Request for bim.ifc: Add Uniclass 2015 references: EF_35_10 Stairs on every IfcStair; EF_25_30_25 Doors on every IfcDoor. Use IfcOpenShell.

First a look at what the model holds.

```python
import ifcopenshell

model = ifcopenshell.open("bim.ifc")
print(model.schema)
print("classifications:", [c.Name for c in model.by_type("IfcClassification")])
for ifc_class in ("IfcDoor", "IfcRoof", "IfcStair", "IfcWall", "IfcWindow"):
    print(ifc_class, len(model.by_type(ifc_class)))
```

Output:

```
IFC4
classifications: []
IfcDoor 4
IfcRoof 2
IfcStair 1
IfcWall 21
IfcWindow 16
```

```python
import ifcopenshell
import ifcopenshell.api.classification

model = ifcopenshell.open("bim.ifc")

system = ifcopenshell.api.classification.add_classification(model, classification="Uniclass 2015")

codes = {
    "IfcStair": ("EF_35_10", "Stairs"),
    "IfcDoor": ("EF_25_30_25", "Doors"),
}
for ifc_class, (code, name) in codes.items():
    products = model.by_type(ifc_class)
    ifcopenshell.api.classification.add_reference(
        model, products=products, classification=system, identification=code, name=name
    )
    print(code, len(products))

model.write("bim_updated.ifc")
```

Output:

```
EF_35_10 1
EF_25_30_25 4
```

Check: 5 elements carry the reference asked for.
